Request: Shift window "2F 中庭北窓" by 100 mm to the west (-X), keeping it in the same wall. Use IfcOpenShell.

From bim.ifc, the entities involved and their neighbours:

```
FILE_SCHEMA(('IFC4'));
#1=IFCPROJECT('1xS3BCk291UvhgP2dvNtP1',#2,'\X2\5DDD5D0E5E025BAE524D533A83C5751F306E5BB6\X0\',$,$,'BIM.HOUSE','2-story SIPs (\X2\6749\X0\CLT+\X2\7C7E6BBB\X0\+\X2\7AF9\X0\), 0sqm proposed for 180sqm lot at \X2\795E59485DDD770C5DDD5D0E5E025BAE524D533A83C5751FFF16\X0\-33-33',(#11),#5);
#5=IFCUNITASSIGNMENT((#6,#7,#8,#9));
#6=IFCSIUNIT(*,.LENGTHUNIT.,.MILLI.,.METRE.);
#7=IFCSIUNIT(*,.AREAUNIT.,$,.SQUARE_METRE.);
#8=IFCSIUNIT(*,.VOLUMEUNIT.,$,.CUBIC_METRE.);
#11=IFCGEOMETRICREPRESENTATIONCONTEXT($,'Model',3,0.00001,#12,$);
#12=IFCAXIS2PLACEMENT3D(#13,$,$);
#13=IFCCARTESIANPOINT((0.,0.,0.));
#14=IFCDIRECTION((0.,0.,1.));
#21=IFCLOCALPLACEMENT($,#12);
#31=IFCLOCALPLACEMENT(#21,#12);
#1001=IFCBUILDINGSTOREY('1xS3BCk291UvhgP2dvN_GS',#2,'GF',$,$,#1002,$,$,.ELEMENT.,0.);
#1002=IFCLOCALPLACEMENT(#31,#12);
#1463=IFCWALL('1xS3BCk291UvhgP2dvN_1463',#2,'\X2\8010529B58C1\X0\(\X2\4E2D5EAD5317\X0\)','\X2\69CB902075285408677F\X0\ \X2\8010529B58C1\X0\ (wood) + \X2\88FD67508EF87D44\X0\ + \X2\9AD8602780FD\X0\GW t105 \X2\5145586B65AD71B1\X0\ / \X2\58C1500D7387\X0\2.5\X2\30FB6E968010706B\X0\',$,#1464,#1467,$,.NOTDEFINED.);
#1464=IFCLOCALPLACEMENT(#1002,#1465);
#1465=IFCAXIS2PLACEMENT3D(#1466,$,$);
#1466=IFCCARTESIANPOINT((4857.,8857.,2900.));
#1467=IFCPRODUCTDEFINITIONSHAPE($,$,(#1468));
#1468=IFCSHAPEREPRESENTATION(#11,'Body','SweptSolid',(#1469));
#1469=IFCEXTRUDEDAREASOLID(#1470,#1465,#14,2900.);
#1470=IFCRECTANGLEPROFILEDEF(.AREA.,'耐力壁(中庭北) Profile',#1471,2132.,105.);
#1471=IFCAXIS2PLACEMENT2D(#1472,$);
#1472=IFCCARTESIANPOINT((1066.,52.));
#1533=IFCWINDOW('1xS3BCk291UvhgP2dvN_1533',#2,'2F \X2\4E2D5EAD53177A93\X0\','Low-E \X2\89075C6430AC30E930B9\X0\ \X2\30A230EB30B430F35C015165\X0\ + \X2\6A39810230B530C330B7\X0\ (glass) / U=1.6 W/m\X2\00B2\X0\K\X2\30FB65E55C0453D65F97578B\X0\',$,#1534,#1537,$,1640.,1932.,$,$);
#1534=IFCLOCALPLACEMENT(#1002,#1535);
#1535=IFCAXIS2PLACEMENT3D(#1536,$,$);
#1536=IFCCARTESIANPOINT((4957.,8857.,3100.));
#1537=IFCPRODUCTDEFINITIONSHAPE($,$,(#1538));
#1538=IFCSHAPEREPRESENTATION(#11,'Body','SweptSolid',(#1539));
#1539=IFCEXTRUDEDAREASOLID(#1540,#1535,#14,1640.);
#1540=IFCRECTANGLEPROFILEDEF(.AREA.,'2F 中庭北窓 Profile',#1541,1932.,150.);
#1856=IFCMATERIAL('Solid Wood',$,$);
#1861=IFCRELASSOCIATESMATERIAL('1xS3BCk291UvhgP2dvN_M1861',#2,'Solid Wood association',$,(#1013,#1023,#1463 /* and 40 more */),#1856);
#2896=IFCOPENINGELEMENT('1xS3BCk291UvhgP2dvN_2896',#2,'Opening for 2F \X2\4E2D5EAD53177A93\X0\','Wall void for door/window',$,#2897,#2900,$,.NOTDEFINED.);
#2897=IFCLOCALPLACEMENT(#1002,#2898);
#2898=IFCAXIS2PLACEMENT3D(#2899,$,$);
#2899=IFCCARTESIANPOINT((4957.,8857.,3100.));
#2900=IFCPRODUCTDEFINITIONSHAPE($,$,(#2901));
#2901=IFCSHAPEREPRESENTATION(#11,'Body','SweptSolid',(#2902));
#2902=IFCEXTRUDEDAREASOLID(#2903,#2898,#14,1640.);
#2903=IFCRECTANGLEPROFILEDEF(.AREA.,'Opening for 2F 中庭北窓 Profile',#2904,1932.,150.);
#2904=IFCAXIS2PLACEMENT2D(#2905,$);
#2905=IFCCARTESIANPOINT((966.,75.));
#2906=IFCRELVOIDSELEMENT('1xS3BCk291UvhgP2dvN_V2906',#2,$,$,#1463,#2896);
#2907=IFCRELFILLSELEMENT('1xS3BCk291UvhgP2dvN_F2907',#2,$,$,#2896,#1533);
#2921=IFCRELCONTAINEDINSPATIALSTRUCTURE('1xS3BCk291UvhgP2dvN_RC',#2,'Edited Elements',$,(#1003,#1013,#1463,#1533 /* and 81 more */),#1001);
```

```python
import ifcopenshell
import ifcopenshell.api.geometry
import ifcopenshell.util.placement
import ifcopenshell.util.unit

model = ifcopenshell.open("bim.ifc")
unit_scale = ifcopenshell.util.unit.calculate_unit_scale(model)

window = model.by_guid("1xS3BCk291UvhgP2dvN_1533")
opening = window.FillsVoids[0].RelatingOpeningElement
wall = opening.VoidsElements[0].RelatingBuildingElement

wall_matrix = ifcopenshell.util.placement.get_local_placement(wall.ObjectPlacement)
shift = wall_matrix[:3, 0] * -0.1 / unit_scale
before = ifcopenshell.util.placement.get_local_placement(window.ObjectPlacement)[:3, 3].copy()

# The window is not placed relative to its opening, so move both.
for product in (opening, window):
    matrix = ifcopenshell.util.placement.get_local_placement(product.ObjectPlacement)
    matrix[:3, 3] += shift
    ifcopenshell.api.geometry.edit_object_placement(model, product=product, matrix=matrix, is_si=False)

after = ifcopenshell.util.placement.get_local_placement(window.ObjectPlacement)[:3, 3]
print("window moved by", (after - before).round(3) + 0.0)

model.write("bim_v2.ifc")
```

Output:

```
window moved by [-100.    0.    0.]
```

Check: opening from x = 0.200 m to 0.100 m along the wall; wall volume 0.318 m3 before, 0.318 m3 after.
